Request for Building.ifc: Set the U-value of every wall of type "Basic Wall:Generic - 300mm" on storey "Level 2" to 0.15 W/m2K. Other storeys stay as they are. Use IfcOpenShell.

First a look at what the model holds.

```python
import ifcopenshell
import ifcopenshell.util.element

model = ifcopenshell.open("Building.ifc")
print(model.schema)
storey = next(s for s in model.by_type("IfcBuildingStorey") if s.Name == "Level 2")
walls = [e for e in ifcopenshell.util.element.get_decomposition(storey) if e.is_a("IfcWall")]
seen = {}
for e in walls:
    element_type = ifcopenshell.util.element.get_type(e)
    key = (element_type.Name if element_type != e and element_type else None, ifcopenshell.util.element.get_pset(e, "Pset_WallCommon", "ThermalTransmittance"))
    seen[key] = seen.get(key, 0) + 1
for (name, value), count in sorted(seen.items(), key=str):
    print(count, "x", name, "|", value)
```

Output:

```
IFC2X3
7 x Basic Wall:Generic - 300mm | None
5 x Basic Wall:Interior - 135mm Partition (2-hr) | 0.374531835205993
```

```python
import ifcopenshell
import ifcopenshell.api.pset
import ifcopenshell.util.element

model = ifcopenshell.open("Building.ifc")

storey = next(s for s in model.by_type("IfcBuildingStorey") if s.Name == "Level 2")
walls = [e for e in ifcopenshell.util.element.get_decomposition(storey) if e.is_a("IfcWall")]

count = 0
for e in walls:
    element_type = ifcopenshell.util.element.get_type(e)
    if element_type in (None, e) or element_type.Name != "Basic Wall:Generic - 300mm":
        continue
    # add_pset returns the element's existing set when there is one.
    pset = ifcopenshell.api.pset.add_pset(model, product=e, name="Pset_WallCommon")
    ifcopenshell.api.pset.edit_pset(model, pset=pset, properties={"ThermalTransmittance": 0.15})
    count += 1

print(count, "walls updated")

model.write("Building_v2.ifc")
```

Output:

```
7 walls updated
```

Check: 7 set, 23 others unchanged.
